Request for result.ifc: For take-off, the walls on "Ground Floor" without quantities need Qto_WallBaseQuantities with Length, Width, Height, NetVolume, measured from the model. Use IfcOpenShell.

First a look at what the model holds.

```python
import ifcopenshell
import ifcopenshell.util.element
import ifcopenshell.util.unit

model = ifcopenshell.open("result.ifc")
print(model.schema)
for unit_type in ("LENGTHUNIT", "AREAUNIT", "VOLUMEUNIT"):
    print(unit_type, ifcopenshell.util.unit.calculate_unit_scale(model, unit_type))
storey = next(s for s in model.by_type("IfcBuildingStorey") if s.Name == "Ground Floor")
walls = [e for e in ifcopenshell.util.element.get_decomposition(storey) if e.is_a("IfcWall")]
for e in sorted(walls, key=lambda e: e.id()):
    print(e.id(), e.is_a(), e.Name, list(ifcopenshell.util.element.get_psets(e, qtos_only=True)), sep=" | ")
```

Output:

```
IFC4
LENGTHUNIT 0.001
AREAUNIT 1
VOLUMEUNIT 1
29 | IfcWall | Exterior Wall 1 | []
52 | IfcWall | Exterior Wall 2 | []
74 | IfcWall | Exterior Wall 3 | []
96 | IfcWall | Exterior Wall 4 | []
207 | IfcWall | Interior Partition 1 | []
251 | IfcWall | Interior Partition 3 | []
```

```python
import ifcopenshell
import ifcopenshell.api.pset
import ifcopenshell.geom
import ifcopenshell.util.element
import ifcopenshell.util.shape
import ifcopenshell.util.unit

model = ifcopenshell.open("result.ifc")
unit_scale = ifcopenshell.util.unit.calculate_unit_scale(model)
volume_scale = ifcopenshell.util.unit.calculate_unit_scale(model, "VOLUMEUNIT")
settings = ifcopenshell.geom.settings()

storey = next(s for s in model.by_type("IfcBuildingStorey") if s.Name == "Ground Floor")
walls = [e for e in ifcopenshell.util.element.get_decomposition(storey) if e.is_a("IfcWall")]

for e in sorted(walls, key=lambda e: e.id()):
    if ifcopenshell.util.element.get_psets(e, qtos_only=True, should_inherit=False):
        continue
    # Geometry comes back in metres, in the element's own axes.
    shape = ifcopenshell.geom.create_shape(settings, e)
    values = {
        "Length": ifcopenshell.util.shape.get_x(shape.geometry) / unit_scale,
        "Width": ifcopenshell.util.shape.get_y(shape.geometry) / unit_scale,
        "Height": ifcopenshell.util.shape.get_z(shape.geometry) / unit_scale,
        "NetVolume": ifcopenshell.util.shape.get_volume(shape.geometry) / volume_scale,
    }
    qto = ifcopenshell.api.pset.add_qto(model, product=e, name="Qto_WallBaseQuantities")
    ifcopenshell.api.pset.edit_qto(model, qto=qto, properties=values)
    print(e.id(), {k: round(v, 3) for k, v in values.items()})

model.write("result_edited.ifc")
```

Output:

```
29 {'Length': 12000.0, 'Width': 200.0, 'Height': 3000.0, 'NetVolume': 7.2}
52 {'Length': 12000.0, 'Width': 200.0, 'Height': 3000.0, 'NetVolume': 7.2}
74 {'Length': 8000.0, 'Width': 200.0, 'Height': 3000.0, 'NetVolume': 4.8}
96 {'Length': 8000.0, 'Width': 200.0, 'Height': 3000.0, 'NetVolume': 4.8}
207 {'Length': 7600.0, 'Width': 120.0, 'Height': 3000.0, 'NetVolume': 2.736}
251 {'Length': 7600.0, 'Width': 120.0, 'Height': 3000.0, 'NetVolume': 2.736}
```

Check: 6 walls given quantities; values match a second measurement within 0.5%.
